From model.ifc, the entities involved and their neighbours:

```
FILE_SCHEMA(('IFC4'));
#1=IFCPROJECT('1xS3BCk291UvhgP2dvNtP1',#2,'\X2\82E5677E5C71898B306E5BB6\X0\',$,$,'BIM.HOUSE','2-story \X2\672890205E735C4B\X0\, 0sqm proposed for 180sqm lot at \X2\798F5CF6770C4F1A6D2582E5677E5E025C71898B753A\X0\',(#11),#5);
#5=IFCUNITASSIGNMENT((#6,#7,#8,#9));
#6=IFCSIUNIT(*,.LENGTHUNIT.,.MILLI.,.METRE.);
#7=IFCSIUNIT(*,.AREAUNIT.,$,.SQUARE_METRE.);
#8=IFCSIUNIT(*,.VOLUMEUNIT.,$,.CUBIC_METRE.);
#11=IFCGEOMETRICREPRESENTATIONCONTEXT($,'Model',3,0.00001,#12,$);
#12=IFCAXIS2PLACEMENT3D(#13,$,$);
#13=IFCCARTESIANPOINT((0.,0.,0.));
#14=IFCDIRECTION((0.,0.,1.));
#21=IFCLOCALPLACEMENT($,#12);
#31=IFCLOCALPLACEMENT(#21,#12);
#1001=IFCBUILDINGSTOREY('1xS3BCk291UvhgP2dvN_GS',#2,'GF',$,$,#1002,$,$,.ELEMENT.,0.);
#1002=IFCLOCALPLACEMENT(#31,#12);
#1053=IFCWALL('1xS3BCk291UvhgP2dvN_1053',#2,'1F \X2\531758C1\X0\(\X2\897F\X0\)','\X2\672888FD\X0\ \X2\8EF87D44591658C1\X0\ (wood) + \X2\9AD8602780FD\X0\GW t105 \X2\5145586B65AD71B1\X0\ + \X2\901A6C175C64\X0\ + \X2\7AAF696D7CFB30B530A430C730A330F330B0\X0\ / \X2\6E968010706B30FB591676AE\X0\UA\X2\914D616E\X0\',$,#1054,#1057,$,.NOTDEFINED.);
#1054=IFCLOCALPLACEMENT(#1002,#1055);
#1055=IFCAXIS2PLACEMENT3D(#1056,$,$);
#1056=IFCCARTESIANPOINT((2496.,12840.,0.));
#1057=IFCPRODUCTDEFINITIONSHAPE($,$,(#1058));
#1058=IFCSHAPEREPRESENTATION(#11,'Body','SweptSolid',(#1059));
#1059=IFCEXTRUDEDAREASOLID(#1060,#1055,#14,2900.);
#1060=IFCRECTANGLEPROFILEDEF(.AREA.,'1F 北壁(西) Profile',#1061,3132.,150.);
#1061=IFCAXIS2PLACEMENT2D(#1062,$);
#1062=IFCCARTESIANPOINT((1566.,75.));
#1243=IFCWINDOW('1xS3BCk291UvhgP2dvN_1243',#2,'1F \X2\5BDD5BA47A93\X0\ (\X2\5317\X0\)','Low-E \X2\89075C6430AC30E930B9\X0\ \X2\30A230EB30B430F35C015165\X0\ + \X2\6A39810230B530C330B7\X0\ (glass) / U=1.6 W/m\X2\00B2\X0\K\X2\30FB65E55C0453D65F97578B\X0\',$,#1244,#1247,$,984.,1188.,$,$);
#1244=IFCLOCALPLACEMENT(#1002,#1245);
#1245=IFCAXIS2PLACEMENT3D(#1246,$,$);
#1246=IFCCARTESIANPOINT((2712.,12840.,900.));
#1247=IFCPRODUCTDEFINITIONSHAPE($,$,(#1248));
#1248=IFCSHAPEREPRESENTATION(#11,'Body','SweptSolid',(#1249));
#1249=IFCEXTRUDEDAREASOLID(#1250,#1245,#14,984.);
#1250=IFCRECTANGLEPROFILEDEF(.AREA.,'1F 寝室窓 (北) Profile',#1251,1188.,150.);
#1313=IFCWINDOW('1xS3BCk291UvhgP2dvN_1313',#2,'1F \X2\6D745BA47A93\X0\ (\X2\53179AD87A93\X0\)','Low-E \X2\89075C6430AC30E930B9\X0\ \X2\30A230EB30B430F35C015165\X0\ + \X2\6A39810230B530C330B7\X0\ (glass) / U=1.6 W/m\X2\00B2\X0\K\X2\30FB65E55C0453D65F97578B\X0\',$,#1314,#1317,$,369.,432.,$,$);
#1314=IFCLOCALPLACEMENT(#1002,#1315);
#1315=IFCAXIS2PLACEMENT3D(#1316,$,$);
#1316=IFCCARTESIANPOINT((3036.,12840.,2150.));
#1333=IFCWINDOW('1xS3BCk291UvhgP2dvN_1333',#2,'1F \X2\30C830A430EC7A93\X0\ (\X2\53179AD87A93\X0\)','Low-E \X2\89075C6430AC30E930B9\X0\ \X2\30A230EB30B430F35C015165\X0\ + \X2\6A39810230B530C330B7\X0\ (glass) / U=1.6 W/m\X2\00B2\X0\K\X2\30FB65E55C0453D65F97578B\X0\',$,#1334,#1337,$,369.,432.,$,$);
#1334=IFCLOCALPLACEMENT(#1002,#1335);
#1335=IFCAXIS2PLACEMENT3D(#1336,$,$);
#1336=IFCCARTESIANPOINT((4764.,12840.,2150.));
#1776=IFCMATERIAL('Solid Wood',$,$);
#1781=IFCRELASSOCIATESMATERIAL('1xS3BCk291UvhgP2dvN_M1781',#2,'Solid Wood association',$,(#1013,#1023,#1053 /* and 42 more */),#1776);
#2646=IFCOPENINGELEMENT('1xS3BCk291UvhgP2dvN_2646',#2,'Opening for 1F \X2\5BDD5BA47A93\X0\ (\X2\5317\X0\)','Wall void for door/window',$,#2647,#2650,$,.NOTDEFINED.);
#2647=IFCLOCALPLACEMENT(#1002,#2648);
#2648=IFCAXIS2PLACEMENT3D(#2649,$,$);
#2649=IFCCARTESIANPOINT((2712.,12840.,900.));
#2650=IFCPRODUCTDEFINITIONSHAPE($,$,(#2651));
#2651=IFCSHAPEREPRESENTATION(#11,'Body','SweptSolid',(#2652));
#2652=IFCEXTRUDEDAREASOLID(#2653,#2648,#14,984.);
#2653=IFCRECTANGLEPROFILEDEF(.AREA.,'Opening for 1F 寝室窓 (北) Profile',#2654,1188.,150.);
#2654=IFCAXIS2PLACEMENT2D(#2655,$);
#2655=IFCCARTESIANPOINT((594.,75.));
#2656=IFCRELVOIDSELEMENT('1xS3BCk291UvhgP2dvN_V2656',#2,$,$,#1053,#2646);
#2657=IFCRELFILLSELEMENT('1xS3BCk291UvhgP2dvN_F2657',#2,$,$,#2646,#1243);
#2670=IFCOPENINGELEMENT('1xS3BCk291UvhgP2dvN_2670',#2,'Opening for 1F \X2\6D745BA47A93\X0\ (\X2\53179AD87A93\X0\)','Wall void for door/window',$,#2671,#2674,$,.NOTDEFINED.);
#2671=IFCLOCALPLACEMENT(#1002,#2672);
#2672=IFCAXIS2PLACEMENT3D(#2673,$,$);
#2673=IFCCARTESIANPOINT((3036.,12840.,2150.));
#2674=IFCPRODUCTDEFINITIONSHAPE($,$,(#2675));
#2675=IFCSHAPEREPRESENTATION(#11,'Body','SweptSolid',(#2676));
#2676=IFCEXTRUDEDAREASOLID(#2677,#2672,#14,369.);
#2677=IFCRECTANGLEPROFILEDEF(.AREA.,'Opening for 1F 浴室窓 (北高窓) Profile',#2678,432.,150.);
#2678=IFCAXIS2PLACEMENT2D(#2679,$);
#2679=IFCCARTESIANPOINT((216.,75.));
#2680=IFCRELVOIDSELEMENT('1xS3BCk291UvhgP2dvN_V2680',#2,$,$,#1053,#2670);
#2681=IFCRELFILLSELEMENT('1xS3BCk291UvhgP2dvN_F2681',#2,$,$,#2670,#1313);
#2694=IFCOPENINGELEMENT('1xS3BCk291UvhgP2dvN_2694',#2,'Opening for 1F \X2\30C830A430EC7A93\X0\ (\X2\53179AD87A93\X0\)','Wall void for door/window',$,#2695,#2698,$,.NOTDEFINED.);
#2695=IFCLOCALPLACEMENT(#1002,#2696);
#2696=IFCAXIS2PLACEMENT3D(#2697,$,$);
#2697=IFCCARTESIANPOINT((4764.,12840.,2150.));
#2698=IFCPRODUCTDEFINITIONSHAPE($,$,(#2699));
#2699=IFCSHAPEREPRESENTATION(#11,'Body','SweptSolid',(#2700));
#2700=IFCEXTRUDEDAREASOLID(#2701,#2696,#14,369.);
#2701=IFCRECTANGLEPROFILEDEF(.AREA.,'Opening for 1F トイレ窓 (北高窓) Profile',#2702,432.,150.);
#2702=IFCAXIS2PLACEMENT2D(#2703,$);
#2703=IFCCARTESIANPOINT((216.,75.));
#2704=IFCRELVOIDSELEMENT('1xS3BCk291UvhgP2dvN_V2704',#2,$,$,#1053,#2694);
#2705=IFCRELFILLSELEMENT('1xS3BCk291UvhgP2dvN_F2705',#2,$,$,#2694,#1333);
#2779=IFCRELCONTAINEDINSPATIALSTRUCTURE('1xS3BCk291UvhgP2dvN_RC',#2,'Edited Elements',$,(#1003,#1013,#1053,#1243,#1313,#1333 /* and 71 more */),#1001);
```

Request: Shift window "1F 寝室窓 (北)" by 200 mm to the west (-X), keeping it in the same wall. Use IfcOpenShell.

```python
import ifcopenshell
import ifcopenshell.api.geometry
import ifcopenshell.util.placement
import ifcopenshell.util.unit

model = ifcopenshell.open("model.ifc")
unit_scale = ifcopenshell.util.unit.calculate_unit_scale(model)

window = model.by_guid("1xS3BCk291UvhgP2dvN_1243")
opening = window.FillsVoids[0].RelatingOpeningElement
wall = opening.VoidsElements[0].RelatingBuildingElement

wall_matrix = ifcopenshell.util.placement.get_local_placement(wall.ObjectPlacement)
shift = wall_matrix[:3, 0] * -0.2 / unit_scale
before = ifcopenshell.util.placement.get_local_placement(window.ObjectPlacement)[:3, 3].copy()

# The window is not placed relative to its opening, so move both.
for product in (opening, window):
    matrix = ifcopenshell.util.placement.get_local_placement(product.ObjectPlacement)
    matrix[:3, 3] += shift
    ifcopenshell.api.geometry.edit_object_placement(model, product=product, matrix=matrix, is_si=False)

after = ifcopenshell.util.placement.get_local_placement(window.ObjectPlacement)[:3, 3]
print("window moved by", (after - before).round(3) + 0.0)

model.write("model_rev.ifc")
```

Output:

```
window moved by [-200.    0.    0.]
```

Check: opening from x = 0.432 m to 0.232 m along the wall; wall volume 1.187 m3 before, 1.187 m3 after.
